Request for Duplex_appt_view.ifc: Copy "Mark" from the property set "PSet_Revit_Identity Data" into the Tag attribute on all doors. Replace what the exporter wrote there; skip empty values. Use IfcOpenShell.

First a look at what the model holds.

```python
import ifcopenshell
import ifcopenshell.util.element

model = ifcopenshell.open("Duplex_appt_view.ifc")
print(model.schema)
doors = model.by_type("IfcDoor")
print(len(doors), "doors")
for e in doors[:8]:
    source = ifcopenshell.util.element.get_pset(e, "PSet_Revit_Identity Data", "Mark")
    target = e.Tag
    print(e.id(), repr(source), repr(target), sep=" | ")
```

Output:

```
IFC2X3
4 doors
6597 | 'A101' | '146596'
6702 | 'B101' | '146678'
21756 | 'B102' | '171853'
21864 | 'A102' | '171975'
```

```python
import ifcopenshell
import ifcopenshell.util.element

model = ifcopenshell.open("Duplex_appt_view.ifc")

count = 0
for e in model.by_type("IfcDoor"):
    value = ifcopenshell.util.element.get_pset(e, "PSet_Revit_Identity Data", "Mark")
    current = e.Tag
    if not value or not value.strip() or current == value:
        continue
    e.Tag = value
    count += 1

print(count, "doors updated")

model.write("Duplex_appt_view_rev.ifc")
```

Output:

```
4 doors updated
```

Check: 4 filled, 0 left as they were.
